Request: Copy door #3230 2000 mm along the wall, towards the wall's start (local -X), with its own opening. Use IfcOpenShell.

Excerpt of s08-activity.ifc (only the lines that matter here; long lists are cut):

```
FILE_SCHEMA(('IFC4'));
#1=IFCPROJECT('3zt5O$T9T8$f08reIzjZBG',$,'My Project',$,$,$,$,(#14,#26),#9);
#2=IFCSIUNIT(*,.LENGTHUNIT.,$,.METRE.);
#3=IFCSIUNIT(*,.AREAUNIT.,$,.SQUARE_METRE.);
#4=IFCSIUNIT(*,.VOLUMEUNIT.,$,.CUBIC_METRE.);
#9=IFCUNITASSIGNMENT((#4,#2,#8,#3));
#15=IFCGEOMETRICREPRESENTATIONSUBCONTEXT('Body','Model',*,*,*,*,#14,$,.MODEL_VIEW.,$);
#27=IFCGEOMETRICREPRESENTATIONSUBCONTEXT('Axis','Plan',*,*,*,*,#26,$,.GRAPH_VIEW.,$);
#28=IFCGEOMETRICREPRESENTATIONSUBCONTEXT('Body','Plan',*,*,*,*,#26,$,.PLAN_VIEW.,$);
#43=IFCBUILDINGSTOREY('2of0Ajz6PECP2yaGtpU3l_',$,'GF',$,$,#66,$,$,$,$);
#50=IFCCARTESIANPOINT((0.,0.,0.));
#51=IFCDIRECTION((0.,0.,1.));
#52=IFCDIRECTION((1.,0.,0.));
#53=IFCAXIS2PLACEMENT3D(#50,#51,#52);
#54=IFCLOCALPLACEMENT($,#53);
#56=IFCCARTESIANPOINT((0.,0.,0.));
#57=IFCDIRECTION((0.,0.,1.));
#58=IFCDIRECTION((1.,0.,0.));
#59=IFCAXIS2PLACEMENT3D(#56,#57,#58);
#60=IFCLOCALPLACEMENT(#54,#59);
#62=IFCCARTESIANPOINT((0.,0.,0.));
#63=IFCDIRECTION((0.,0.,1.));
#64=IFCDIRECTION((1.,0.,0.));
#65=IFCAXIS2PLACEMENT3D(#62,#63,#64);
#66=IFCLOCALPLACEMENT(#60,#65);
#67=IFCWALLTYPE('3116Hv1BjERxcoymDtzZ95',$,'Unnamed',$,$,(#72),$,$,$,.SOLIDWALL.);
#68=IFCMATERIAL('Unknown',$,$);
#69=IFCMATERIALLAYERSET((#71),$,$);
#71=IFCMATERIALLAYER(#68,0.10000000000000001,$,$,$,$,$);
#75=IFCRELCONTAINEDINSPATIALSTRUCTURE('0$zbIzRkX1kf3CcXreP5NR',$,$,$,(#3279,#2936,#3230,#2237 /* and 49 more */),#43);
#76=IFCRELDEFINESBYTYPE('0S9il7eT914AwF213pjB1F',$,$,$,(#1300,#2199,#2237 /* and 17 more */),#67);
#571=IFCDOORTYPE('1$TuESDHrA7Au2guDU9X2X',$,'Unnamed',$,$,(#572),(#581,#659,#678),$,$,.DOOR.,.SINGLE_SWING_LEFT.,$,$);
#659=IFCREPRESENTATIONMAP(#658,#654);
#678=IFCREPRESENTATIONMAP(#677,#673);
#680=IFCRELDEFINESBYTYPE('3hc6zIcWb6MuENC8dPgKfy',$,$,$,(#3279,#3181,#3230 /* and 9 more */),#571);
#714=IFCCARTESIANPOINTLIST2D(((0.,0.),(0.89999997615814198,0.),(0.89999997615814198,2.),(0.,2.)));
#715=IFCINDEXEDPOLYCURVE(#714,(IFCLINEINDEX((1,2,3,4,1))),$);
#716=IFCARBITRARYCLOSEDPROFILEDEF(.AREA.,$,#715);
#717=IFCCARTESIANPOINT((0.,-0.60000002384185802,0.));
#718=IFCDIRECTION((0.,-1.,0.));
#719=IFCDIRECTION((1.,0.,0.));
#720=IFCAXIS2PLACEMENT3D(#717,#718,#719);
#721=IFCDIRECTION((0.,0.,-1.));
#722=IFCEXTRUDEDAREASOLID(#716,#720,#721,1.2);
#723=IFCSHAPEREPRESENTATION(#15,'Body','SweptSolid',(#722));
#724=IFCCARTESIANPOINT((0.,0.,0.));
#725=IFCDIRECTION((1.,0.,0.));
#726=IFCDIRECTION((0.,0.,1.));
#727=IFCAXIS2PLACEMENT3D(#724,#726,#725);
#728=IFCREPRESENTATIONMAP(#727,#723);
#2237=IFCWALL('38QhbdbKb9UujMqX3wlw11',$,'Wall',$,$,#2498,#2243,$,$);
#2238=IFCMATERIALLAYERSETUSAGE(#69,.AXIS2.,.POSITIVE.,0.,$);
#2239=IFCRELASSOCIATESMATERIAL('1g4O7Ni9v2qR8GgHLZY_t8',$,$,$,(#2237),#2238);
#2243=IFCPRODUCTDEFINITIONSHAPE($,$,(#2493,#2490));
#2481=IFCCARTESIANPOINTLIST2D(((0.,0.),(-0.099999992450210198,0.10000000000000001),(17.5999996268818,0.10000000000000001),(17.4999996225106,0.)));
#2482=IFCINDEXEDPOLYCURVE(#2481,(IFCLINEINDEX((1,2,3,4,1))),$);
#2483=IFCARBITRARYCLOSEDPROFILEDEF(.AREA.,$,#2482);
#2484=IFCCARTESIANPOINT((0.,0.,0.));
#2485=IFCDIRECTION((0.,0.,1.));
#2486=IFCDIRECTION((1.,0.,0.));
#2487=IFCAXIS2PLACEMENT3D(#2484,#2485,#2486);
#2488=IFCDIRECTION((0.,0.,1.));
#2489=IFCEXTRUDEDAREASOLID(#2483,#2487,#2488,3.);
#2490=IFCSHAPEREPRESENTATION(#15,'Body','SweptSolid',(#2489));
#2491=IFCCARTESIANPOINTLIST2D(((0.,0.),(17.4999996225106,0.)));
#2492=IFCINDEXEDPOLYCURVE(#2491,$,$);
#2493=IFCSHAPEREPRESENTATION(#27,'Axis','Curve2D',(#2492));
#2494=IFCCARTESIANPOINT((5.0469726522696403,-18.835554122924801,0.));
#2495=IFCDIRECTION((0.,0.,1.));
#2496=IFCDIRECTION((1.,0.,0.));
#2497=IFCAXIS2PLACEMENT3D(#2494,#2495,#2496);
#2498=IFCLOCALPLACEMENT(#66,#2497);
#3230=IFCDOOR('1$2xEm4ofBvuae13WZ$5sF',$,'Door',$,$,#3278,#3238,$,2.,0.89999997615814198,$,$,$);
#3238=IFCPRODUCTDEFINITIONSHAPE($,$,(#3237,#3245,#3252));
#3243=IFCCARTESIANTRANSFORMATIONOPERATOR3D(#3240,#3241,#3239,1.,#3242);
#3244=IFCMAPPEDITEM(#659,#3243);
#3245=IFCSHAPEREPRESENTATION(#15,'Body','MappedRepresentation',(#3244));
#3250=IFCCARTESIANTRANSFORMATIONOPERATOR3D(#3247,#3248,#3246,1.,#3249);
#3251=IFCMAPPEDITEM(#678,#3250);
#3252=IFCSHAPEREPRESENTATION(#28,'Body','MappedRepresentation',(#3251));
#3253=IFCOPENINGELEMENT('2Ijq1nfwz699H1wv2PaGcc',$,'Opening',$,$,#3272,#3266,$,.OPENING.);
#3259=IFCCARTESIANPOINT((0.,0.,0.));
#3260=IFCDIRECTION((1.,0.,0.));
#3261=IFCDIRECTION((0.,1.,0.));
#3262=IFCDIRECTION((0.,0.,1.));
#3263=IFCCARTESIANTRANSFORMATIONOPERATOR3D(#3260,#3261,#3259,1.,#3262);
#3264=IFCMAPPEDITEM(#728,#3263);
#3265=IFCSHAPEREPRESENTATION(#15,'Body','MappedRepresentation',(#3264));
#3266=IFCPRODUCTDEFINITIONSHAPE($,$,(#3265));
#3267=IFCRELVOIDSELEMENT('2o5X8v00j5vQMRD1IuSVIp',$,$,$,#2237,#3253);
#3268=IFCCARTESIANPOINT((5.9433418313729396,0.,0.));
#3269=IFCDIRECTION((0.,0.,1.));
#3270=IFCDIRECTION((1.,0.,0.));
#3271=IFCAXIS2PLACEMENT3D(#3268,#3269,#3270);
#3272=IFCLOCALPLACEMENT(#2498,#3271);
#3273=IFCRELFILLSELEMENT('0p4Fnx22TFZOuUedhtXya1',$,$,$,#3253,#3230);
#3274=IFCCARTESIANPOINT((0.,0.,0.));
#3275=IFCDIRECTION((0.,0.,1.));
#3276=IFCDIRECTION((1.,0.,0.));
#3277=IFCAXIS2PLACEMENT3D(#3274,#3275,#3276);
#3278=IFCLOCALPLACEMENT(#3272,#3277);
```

```python
import ifcopenshell
import ifcopenshell.api.feature
import ifcopenshell.api.geometry
import ifcopenshell.api.root
import ifcopenshell.geom
import ifcopenshell.util.element
import ifcopenshell.util.placement
import ifcopenshell.util.shape
import ifcopenshell.util.unit

model = ifcopenshell.open("s08-activity.ifc")
unit_scale = ifcopenshell.util.unit.calculate_unit_scale(model)
settings = ifcopenshell.geom.settings()


def volume(element):
    """Net volume in cubic metres, openings subtracted."""
    shape = ifcopenshell.geom.create_shape(settings, element)
    return ifcopenshell.util.shape.get_volume(shape.geometry)


door = model.by_guid("1$2xEm4ofBvuae13WZ$5sF")
opening = door.FillsVoids[0].RelatingOpeningElement
wall = opening.VoidsElements[0].RelatingBuildingElement
before = volume(wall)
shift = ifcopenshell.util.placement.get_local_placement(wall.ObjectPlacement)[:3, 0] * -2 / unit_scale

# copy_class copies the void relationship, type, container and properties, but no geometry.
new_opening = ifcopenshell.api.root.copy_class(model, product=opening)
new_opening.Representation = ifcopenshell.util.element.copy_deep(
    model, opening.Representation, exclude=["IfcGeometricRepresentationContext", "IfcRepresentationMap"]
)
new_door = ifcopenshell.api.root.copy_class(model, product=door)
new_door.Representation = ifcopenshell.util.element.copy_deep(
    model, door.Representation, exclude=["IfcGeometricRepresentationContext", "IfcRepresentationMap"]
)
ifcopenshell.api.feature.add_filling(model, opening=new_opening, element=new_door)

for old, new in ((opening, new_opening), (door, new_door)):
    matrix = ifcopenshell.util.placement.get_local_placement(old.ObjectPlacement)
    matrix[:3, 3] += shift
    ifcopenshell.api.geometry.edit_object_placement(model, product=new, matrix=matrix, is_si=False)

after = volume(wall)

print(f"wall volume {before:.3f} -> {after:.3f} m3")

model.write("s08-activity_rev.ifc")
```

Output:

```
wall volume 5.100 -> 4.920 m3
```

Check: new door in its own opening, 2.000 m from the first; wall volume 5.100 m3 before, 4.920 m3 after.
